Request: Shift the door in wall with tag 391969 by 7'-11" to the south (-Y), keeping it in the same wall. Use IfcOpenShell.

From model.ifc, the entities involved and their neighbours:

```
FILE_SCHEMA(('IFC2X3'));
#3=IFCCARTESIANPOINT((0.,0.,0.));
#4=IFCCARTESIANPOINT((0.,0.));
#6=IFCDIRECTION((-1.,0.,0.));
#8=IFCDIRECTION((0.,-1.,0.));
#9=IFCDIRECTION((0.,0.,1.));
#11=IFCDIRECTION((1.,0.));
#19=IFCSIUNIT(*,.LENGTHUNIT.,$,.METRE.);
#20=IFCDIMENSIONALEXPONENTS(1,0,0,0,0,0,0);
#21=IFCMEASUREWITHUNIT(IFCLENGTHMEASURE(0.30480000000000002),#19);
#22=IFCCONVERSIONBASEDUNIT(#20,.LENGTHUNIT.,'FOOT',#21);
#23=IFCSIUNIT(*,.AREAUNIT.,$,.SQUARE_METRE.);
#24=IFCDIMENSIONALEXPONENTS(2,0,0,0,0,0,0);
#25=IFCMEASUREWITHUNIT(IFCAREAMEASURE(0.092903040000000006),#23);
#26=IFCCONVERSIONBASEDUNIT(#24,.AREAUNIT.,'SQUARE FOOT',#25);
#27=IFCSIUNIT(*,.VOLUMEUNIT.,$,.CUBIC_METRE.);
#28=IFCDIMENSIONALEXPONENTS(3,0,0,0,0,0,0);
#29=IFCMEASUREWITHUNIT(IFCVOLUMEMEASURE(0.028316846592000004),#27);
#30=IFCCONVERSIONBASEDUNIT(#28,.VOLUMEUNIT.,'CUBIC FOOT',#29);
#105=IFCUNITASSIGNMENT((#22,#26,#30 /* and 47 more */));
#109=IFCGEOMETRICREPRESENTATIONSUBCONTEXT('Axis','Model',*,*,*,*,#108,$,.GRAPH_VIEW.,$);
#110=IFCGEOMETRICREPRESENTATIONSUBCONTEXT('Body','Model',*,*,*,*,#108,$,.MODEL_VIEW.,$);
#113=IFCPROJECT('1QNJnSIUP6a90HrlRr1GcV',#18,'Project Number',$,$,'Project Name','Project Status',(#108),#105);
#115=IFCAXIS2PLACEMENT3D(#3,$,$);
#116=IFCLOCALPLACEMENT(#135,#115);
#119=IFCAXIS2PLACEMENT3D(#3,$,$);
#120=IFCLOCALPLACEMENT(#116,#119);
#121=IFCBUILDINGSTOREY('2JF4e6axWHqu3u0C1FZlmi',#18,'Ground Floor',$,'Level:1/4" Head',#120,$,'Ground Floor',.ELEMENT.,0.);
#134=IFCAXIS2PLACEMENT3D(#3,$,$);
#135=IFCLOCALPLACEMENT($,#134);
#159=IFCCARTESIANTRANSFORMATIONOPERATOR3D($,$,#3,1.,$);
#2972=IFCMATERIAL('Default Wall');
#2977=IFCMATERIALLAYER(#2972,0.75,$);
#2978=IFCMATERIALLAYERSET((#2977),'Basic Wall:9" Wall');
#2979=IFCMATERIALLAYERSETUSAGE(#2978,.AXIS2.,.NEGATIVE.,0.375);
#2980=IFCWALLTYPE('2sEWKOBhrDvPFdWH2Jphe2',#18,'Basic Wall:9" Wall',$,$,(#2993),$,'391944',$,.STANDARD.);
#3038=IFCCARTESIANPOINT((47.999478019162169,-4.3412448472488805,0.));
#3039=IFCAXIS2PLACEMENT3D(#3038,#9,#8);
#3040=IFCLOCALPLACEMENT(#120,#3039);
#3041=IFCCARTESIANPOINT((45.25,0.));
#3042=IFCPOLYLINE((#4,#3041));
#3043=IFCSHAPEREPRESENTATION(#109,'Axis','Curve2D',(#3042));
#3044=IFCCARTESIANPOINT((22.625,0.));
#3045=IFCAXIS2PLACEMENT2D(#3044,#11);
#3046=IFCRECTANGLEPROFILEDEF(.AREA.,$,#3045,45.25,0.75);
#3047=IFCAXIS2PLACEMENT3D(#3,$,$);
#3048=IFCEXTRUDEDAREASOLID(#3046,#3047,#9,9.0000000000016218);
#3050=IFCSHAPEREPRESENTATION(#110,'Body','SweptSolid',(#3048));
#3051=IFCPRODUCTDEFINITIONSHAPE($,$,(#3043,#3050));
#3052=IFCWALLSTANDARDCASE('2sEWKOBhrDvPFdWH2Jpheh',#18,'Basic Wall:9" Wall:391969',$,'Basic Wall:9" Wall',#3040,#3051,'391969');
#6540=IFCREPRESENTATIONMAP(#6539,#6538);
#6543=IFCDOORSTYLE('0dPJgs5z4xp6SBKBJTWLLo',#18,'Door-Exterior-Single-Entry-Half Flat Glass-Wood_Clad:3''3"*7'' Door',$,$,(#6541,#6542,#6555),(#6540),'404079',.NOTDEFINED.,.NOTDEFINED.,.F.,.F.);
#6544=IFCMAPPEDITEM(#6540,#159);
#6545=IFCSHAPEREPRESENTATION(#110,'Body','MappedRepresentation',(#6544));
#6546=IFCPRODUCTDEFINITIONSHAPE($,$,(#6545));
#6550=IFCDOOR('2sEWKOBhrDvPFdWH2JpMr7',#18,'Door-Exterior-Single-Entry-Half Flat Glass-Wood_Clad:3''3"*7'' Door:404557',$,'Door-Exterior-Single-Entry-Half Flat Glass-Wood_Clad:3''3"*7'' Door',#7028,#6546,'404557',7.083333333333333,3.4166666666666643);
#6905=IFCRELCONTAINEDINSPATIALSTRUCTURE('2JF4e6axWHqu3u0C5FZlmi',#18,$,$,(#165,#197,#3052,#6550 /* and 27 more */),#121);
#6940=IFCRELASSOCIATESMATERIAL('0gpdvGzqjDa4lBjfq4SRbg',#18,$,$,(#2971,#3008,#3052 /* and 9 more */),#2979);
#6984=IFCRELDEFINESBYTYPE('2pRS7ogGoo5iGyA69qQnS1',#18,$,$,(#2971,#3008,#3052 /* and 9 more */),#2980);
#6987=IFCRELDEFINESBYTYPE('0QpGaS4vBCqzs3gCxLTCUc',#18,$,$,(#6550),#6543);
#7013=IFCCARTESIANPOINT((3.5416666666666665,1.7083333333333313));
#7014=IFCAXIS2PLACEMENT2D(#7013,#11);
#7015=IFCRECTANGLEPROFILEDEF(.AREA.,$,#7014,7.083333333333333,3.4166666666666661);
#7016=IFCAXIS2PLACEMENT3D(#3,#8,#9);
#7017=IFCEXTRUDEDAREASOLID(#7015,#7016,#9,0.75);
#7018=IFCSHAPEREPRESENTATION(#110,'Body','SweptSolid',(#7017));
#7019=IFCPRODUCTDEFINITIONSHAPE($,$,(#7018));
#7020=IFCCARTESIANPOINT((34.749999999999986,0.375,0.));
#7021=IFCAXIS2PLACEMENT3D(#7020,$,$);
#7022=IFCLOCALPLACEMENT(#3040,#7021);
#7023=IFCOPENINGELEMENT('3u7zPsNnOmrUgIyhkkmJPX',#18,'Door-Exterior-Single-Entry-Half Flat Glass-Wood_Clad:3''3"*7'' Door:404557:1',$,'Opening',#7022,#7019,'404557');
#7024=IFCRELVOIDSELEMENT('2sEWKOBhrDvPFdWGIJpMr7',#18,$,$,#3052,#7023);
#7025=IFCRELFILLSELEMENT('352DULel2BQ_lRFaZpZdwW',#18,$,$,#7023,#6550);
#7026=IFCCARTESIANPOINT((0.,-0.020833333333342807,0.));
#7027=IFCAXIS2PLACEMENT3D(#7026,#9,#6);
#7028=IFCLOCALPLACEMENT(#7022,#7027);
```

```python
import ifcopenshell
import ifcopenshell.api.geometry
import ifcopenshell.util.placement
import ifcopenshell.util.unit

model = ifcopenshell.open("model.ifc")
unit_scale = ifcopenshell.util.unit.calculate_unit_scale(model)

door = model.by_guid("2sEWKOBhrDvPFdWH2JpMr7")
opening = door.FillsVoids[0].RelatingOpeningElement
wall = opening.VoidsElements[0].RelatingBuildingElement

wall_matrix = ifcopenshell.util.placement.get_local_placement(wall.ObjectPlacement)
shift = wall_matrix[:3, 0] * 95 * 0.0254 / unit_scale
before = ifcopenshell.util.placement.get_local_placement(door.ObjectPlacement)[:3, 3].copy()

# The door is placed relative to its opening, so it follows when the opening moves.
matrix = ifcopenshell.util.placement.get_local_placement(opening.ObjectPlacement)
matrix[:3, 3] += shift
ifcopenshell.api.geometry.edit_object_placement(
    model, product=opening, matrix=matrix, is_si=False, should_transform_children=True
)

after = ifcopenshell.util.placement.get_local_placement(door.ObjectPlacement)[:3, 3]
print("door moved by", (after - before).round(3) + 0.0)

model.write("model_edited.ifc")
```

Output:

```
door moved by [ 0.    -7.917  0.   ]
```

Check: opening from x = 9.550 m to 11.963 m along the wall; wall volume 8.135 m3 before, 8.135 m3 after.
